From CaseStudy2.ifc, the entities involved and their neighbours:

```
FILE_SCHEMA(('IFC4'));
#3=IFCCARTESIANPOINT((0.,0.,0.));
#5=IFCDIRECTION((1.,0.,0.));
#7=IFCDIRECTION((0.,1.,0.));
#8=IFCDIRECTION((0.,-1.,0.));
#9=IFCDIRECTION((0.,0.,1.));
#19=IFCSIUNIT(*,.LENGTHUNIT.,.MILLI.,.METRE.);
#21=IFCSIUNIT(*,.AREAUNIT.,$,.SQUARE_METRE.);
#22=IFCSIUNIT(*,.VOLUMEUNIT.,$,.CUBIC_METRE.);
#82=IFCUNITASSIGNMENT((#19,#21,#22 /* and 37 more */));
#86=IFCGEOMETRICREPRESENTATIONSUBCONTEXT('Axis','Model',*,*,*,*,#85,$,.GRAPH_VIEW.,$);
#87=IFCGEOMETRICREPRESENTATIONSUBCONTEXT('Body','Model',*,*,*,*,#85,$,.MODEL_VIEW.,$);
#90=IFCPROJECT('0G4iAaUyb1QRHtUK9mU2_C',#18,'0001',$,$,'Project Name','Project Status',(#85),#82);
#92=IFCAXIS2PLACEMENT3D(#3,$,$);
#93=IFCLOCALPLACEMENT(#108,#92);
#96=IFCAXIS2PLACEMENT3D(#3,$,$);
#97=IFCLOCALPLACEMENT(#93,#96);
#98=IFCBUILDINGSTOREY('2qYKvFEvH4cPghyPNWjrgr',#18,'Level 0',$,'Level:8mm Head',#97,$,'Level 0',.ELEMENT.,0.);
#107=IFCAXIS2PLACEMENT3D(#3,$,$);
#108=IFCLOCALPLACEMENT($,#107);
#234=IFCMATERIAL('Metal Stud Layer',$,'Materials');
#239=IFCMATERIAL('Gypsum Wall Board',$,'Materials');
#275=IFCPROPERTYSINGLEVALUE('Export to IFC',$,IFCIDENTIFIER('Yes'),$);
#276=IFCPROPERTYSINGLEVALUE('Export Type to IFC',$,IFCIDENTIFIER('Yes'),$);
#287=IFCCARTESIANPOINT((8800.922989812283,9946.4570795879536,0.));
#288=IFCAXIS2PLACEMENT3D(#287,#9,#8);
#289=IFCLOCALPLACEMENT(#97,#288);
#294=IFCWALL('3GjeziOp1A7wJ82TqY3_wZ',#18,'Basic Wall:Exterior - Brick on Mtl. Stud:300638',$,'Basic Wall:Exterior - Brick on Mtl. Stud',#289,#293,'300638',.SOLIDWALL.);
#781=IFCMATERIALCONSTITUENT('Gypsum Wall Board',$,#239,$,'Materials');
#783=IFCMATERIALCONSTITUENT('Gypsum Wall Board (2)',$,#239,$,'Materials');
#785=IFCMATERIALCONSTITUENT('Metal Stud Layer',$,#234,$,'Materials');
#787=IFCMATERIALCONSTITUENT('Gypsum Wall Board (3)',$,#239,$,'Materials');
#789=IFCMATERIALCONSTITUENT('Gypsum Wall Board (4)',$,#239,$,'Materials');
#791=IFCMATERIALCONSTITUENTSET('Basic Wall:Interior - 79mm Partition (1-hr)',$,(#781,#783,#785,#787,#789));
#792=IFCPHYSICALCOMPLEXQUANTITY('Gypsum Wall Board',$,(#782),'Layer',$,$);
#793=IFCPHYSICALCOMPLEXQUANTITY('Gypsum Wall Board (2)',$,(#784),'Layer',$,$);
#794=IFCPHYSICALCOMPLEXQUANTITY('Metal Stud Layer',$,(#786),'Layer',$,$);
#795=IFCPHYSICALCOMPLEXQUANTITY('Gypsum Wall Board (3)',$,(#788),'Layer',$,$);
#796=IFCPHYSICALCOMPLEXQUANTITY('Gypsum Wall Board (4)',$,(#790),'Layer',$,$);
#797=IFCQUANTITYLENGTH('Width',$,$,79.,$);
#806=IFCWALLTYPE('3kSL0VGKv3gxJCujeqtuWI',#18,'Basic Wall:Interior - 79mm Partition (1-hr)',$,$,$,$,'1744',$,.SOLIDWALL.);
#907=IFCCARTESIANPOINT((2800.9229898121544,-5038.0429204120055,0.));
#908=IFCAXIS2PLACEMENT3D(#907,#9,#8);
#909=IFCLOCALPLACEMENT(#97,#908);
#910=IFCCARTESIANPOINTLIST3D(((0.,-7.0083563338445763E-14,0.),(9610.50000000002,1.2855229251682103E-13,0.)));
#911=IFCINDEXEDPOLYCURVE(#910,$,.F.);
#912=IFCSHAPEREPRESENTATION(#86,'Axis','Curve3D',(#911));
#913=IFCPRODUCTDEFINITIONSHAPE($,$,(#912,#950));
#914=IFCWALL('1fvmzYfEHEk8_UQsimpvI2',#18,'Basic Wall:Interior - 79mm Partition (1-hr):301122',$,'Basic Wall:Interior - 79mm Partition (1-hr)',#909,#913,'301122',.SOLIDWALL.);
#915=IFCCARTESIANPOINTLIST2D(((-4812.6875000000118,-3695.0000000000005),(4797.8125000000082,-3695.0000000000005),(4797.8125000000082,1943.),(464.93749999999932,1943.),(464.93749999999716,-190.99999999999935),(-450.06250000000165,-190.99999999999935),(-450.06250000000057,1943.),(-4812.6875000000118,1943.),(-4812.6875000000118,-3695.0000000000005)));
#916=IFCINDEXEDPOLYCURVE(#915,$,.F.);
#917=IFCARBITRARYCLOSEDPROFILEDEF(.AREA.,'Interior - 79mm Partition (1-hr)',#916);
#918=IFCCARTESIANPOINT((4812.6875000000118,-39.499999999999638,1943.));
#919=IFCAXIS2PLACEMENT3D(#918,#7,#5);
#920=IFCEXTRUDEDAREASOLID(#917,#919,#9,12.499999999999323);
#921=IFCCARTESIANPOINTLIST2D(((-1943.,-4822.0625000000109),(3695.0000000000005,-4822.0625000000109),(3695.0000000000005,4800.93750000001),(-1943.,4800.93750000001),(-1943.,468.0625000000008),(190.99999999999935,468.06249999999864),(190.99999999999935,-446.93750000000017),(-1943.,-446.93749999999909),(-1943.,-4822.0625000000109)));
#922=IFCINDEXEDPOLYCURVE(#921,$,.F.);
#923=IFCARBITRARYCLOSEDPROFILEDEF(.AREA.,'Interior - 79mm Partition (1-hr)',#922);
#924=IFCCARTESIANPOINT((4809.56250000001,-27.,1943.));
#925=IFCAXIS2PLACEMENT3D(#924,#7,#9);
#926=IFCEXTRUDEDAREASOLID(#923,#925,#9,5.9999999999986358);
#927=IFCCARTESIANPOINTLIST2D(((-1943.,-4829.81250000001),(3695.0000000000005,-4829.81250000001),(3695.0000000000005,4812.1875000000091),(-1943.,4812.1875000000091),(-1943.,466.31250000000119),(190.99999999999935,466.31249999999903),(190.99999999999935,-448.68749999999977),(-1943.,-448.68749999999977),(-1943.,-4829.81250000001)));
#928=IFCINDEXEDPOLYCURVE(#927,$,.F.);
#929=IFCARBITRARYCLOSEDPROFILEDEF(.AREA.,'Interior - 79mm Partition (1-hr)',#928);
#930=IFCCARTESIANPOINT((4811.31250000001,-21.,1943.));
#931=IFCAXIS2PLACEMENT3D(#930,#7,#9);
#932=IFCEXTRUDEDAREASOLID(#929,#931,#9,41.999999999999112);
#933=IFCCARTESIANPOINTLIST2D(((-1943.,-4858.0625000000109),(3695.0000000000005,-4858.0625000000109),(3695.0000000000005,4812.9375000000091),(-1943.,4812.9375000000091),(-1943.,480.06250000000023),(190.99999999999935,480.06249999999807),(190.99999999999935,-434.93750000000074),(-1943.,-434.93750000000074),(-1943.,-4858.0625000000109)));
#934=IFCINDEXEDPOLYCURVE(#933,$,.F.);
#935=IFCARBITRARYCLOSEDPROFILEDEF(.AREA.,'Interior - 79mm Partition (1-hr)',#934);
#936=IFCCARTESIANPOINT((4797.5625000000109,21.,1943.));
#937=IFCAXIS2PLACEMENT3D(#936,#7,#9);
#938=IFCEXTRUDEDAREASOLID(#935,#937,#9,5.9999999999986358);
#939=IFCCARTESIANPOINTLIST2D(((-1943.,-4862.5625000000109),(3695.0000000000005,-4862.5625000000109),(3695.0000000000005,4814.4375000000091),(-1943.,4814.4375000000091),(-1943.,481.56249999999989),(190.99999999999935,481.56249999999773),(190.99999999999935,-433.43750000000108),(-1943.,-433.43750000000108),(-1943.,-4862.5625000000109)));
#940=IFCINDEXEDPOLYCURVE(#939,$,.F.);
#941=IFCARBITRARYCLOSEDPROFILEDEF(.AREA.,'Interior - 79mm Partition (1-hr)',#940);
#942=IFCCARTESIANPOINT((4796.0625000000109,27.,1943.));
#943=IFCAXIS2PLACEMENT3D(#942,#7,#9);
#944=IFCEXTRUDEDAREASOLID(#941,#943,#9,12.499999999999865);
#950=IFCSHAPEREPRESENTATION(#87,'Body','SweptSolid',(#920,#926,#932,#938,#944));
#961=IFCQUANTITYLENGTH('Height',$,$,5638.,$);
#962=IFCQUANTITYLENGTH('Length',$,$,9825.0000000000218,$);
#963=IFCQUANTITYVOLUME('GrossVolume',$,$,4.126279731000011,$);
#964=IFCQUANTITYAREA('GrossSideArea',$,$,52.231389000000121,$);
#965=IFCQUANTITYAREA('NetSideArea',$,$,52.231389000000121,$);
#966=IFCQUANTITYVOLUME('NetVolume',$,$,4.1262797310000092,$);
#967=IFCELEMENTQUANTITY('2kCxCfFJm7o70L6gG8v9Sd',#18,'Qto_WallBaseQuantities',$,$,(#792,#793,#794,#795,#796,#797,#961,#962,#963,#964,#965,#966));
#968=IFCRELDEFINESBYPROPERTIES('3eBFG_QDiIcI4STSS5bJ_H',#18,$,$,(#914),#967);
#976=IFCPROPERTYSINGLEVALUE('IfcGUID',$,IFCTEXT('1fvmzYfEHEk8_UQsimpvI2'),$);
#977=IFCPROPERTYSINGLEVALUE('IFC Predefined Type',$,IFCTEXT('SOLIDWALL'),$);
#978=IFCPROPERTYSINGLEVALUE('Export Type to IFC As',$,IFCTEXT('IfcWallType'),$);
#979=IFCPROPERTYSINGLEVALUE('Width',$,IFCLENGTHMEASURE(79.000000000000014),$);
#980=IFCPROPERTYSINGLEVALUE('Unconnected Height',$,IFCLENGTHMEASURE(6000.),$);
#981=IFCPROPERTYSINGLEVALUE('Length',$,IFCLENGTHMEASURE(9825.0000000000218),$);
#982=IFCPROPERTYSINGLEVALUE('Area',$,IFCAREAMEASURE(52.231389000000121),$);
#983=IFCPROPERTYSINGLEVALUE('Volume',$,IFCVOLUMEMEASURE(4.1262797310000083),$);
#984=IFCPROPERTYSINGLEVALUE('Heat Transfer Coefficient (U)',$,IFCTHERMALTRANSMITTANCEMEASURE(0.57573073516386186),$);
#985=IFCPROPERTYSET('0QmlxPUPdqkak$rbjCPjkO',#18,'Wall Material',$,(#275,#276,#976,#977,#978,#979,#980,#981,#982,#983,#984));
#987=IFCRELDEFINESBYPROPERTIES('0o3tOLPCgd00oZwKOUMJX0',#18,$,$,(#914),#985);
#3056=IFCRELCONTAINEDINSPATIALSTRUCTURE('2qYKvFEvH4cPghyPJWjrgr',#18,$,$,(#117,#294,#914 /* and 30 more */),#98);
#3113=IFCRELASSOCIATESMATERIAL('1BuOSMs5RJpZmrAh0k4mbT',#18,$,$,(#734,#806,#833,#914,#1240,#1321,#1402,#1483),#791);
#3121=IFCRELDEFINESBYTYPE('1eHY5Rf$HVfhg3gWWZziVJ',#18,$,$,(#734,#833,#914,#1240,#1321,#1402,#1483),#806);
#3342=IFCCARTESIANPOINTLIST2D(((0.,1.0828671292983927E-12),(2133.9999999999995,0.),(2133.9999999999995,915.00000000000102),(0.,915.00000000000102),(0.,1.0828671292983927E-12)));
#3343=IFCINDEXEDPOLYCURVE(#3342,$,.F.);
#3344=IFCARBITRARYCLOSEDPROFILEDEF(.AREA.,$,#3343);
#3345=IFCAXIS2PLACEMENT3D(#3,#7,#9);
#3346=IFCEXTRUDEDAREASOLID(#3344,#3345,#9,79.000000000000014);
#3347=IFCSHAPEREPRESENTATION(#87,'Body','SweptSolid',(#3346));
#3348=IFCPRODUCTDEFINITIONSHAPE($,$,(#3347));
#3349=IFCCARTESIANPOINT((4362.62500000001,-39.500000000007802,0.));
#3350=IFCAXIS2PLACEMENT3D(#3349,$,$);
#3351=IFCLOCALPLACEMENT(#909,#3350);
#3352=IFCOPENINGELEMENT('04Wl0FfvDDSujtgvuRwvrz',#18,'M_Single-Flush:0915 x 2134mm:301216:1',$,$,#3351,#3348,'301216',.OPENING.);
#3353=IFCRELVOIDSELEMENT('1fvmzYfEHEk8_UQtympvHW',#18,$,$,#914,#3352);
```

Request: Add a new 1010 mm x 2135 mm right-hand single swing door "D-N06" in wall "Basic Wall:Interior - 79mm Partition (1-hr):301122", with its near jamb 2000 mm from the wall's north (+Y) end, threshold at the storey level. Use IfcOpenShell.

```python
import numpy as np
import ifcopenshell
import ifcopenshell.api.feature
import ifcopenshell.api.geometry
import ifcopenshell.api.pset
import ifcopenshell.api.root
import ifcopenshell.api.spatial
import ifcopenshell.geom
import ifcopenshell.util.element
import ifcopenshell.util.placement
import ifcopenshell.util.representation
import ifcopenshell.util.shape
import ifcopenshell.util.unit

model = ifcopenshell.open("CaseStudy2.ifc")
unit_scale = ifcopenshell.util.unit.calculate_unit_scale(model)
area_scale = ifcopenshell.util.unit.calculate_unit_scale(model, "AREAUNIT")
volume_scale = ifcopenshell.util.unit.calculate_unit_scale(model, "VOLUMEUNIT")
settings = ifcopenshell.geom.settings()


def volume(element):
    """Net volume in cubic metres, openings subtracted."""
    shape = ifcopenshell.geom.create_shape(settings, element)
    return ifcopenshell.util.shape.get_volume(shape.geometry)


wall = model.by_guid("1fvmzYfEHEk8_UQsimpvI2")
storey = ifcopenshell.util.element.get_container(wall, ifc_class="IfcBuildingStorey")
context = ifcopenshell.util.representation.get_context(model, "Model", "Body", "MODEL_VIEW")
before = volume(wall)

width, height, from_end, sill = 1.01, 2.135, 2, 0.0  # metres

# The wall runs along its own X axis, and the end named is its -X end.
wall_shape = ifcopenshell.geom.create_shape(settings, wall)
x, y, z = ifcopenshell.util.shape.get_vertices(wall_shape.geometry).T
start = x.min() + from_end
face, thickness = float(y.min()), float(y.max() - y.min())
wall_matrix = ifcopenshell.util.placement.get_local_placement(wall.ObjectPlacement)
level = ifcopenshell.util.placement.get_local_placement(storey.ObjectPlacement)[2, 3]


def in_wall(x, y):
    """Placement at x, y metres in the wall's axes, at sill height."""
    matrix = wall_matrix.copy()
    matrix[:, 3] = wall_matrix @ np.array([x / unit_scale, y / unit_scale, 0.0, 1.0])
    matrix[2, 3] = level + sill / unit_scale
    return matrix


# Opening: a box that overshoots both wall faces by 50 mm.
opening = ifcopenshell.api.root.create_entity(model, ifc_class="IfcOpeningElement", predefined_type="OPENING")
box = ifcopenshell.api.geometry.add_wall_representation(
    model, context=context, length=width, height=height, thickness=thickness + 0.1
)
ifcopenshell.api.geometry.assign_representation(model, product=opening, representation=box)
ifcopenshell.api.geometry.edit_object_placement(model, product=opening, matrix=in_wall(start, face - 0.05), is_si=False)
ifcopenshell.api.feature.add_feature(model, feature=opening, element=wall)

door = ifcopenshell.api.root.create_entity(model, ifc_class="IfcDoor", name="D-N06", predefined_type="DOOR")
door.OverallWidth, door.OverallHeight = width / unit_scale, height / unit_scale
door.OperationType = "SINGLE_SWING_RIGHT"
body = ifcopenshell.api.geometry.add_door_representation(
    model,
    context=context,
    overall_width=door.OverallWidth,
    overall_height=door.OverallHeight,
    operation_type="SINGLE_SWING_RIGHT",
    lining_properties={"LiningDepth": thickness / unit_scale, "ThresholdDepth": thickness / unit_scale},
)
ifcopenshell.api.geometry.assign_representation(model, product=door, representation=body)
ifcopenshell.api.spatial.assign_container(model, products=[door], relating_structure=storey)
ifcopenshell.api.feature.add_filling(model, opening=opening, element=door)

# The lining spans the wall, so the door starts at the wall face.
ifcopenshell.api.geometry.edit_object_placement(model, product=door, matrix=in_wall(start, face), is_si=False)

after = volume(wall)

# Update the wall's stored quantities.
qto = model.by_id(ifcopenshell.util.element.get_pset(wall, "Qto_WallBaseQuantities", should_inherit=False)["id"])
ifcopenshell.api.pset.edit_qto(model, qto=qto, properties={
    "NetSideArea": after / thickness / area_scale,
    "NetVolume": after / volume_scale,
})
pset = model.by_id(ifcopenshell.util.element.get_pset(wall, "Wall Material", should_inherit=False)["id"])
ifcopenshell.api.pset.edit_pset(model, pset=pset, properties={
    "Area": model.create_entity("IfcAreaMeasure", after / thickness / area_scale),
    "Volume": model.create_entity("IfcVolumeMeasure", after / volume_scale),
})

print(f"wall volume {before:.3f} -> {after:.3f} m3")

model.write("CaseStudy2_edited.ifc")
```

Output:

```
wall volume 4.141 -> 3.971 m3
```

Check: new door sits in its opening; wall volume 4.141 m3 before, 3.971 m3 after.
